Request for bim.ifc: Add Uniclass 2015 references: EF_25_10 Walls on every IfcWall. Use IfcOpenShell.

First a look at what the model holds.

```python
import ifcopenshell

model = ifcopenshell.open("bim.ifc")
print(model.schema)
print("classifications:", [c.Name for c in model.by_type("IfcClassification")])
for ifc_class in ("IfcDoor", "IfcRoof", "IfcStair", "IfcWall", "IfcWindow"):
    print(ifc_class, len(model.by_type(ifc_class)))
```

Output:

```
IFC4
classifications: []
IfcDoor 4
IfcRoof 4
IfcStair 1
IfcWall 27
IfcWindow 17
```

```python
import ifcopenshell
import ifcopenshell.api.classification

model = ifcopenshell.open("bim.ifc")

system = ifcopenshell.api.classification.add_classification(model, classification="Uniclass 2015")

codes = {
    "IfcWall": ("EF_25_10", "Walls"),
}
for ifc_class, (code, name) in codes.items():
    products = model.by_type(ifc_class)
    ifcopenshell.api.classification.add_reference(
        model, products=products, classification=system, identification=code, name=name
    )
    print(code, len(products))

model.write("bim-out.ifc")
```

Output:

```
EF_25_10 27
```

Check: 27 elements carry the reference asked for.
